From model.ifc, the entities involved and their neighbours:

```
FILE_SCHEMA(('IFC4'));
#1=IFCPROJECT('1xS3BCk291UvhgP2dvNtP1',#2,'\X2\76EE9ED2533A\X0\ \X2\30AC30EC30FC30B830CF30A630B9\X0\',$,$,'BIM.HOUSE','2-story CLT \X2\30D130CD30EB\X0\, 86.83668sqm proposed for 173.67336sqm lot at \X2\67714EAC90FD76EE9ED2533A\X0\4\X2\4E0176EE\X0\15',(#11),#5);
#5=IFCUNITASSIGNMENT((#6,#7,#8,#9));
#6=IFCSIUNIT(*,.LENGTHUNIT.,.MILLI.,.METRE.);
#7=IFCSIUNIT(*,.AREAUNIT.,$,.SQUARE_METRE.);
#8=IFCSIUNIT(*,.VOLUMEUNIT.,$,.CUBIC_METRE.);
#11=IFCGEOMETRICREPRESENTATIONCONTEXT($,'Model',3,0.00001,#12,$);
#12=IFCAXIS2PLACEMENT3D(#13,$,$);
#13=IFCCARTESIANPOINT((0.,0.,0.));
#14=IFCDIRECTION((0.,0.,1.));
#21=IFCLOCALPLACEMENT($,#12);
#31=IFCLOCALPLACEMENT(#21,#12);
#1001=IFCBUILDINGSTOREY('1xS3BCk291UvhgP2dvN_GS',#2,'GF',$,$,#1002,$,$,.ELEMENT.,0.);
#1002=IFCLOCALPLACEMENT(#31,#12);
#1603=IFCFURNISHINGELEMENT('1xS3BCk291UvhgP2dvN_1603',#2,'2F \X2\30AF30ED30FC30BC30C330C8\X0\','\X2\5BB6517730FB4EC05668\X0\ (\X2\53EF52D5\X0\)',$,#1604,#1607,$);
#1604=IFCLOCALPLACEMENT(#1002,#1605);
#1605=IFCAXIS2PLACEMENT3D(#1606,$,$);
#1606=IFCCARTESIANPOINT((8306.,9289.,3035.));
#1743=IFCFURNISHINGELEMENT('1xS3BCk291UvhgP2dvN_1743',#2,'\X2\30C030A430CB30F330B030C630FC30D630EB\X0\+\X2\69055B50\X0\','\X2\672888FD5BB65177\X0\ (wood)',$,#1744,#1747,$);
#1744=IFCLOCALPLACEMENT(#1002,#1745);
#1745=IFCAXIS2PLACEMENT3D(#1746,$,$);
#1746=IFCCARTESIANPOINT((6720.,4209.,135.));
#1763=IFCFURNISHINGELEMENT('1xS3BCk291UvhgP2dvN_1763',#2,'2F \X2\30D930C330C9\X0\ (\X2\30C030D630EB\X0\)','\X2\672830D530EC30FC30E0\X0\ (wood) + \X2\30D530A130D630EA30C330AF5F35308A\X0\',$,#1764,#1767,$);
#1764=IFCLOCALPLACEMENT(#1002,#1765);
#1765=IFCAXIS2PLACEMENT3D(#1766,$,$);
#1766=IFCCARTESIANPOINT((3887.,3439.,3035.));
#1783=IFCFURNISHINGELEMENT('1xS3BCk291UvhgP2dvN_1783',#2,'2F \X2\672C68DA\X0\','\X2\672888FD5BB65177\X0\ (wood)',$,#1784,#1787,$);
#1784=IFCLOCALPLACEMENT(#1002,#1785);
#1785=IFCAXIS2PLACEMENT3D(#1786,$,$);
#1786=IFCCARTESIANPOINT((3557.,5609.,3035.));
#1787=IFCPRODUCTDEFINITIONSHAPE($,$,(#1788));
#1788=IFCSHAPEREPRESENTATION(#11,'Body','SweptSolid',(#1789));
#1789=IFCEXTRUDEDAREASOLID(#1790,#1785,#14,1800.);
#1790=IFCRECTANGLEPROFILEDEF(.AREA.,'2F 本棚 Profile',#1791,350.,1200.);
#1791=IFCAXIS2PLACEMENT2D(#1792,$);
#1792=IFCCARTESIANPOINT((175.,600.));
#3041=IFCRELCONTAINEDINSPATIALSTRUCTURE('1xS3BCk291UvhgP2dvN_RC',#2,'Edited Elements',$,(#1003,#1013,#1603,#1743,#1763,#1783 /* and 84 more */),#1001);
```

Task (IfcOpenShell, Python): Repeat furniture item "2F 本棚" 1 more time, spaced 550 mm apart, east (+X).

```python
import numpy as np
import ifcopenshell
import ifcopenshell.api.geometry
import ifcopenshell.api.root
import ifcopenshell.util.element
import ifcopenshell.util.placement

model = ifcopenshell.open("model.ifc")


def reuse_history(source, copy):
    """copy_class also copies each property set's owner history, people and application; keep the originals."""
    for rel in copy.IsDefinedBy:
        if rel.is_a("IfcRelDefinesByProperties") and (history := rel.RelatingPropertyDefinition.OwnerHistory):
            rel.RelatingPropertyDefinition.OwnerHistory = source.OwnerHistory
            ifcopenshell.util.element.remove_deep2(model, history)


source = model.by_guid("1xS3BCk291UvhgP2dvN_1783")
base = ifcopenshell.util.placement.get_local_placement(source.ObjectPlacement)
step = np.array([1.0, 0.0, 0.0]) * 550.0

for i in range(1, 2):
    copy = ifcopenshell.api.root.copy_class(model, product=source)
    copy.Representation = ifcopenshell.util.element.copy_deep(
        model, source.Representation, exclude=["IfcGeometricRepresentationContext", "IfcRepresentationMap"]
    )
    reuse_history(source, copy)
    matrix = base.copy()
    matrix[:3, 3] += i * step
    print("added at", matrix[:3, 3].round(3) + 0.0)
    ifcopenshell.api.geometry.edit_object_placement(model, product=copy, matrix=matrix, is_si=False)

model.write("model_edited.ifc")
```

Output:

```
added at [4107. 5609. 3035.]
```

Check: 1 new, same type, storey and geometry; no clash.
